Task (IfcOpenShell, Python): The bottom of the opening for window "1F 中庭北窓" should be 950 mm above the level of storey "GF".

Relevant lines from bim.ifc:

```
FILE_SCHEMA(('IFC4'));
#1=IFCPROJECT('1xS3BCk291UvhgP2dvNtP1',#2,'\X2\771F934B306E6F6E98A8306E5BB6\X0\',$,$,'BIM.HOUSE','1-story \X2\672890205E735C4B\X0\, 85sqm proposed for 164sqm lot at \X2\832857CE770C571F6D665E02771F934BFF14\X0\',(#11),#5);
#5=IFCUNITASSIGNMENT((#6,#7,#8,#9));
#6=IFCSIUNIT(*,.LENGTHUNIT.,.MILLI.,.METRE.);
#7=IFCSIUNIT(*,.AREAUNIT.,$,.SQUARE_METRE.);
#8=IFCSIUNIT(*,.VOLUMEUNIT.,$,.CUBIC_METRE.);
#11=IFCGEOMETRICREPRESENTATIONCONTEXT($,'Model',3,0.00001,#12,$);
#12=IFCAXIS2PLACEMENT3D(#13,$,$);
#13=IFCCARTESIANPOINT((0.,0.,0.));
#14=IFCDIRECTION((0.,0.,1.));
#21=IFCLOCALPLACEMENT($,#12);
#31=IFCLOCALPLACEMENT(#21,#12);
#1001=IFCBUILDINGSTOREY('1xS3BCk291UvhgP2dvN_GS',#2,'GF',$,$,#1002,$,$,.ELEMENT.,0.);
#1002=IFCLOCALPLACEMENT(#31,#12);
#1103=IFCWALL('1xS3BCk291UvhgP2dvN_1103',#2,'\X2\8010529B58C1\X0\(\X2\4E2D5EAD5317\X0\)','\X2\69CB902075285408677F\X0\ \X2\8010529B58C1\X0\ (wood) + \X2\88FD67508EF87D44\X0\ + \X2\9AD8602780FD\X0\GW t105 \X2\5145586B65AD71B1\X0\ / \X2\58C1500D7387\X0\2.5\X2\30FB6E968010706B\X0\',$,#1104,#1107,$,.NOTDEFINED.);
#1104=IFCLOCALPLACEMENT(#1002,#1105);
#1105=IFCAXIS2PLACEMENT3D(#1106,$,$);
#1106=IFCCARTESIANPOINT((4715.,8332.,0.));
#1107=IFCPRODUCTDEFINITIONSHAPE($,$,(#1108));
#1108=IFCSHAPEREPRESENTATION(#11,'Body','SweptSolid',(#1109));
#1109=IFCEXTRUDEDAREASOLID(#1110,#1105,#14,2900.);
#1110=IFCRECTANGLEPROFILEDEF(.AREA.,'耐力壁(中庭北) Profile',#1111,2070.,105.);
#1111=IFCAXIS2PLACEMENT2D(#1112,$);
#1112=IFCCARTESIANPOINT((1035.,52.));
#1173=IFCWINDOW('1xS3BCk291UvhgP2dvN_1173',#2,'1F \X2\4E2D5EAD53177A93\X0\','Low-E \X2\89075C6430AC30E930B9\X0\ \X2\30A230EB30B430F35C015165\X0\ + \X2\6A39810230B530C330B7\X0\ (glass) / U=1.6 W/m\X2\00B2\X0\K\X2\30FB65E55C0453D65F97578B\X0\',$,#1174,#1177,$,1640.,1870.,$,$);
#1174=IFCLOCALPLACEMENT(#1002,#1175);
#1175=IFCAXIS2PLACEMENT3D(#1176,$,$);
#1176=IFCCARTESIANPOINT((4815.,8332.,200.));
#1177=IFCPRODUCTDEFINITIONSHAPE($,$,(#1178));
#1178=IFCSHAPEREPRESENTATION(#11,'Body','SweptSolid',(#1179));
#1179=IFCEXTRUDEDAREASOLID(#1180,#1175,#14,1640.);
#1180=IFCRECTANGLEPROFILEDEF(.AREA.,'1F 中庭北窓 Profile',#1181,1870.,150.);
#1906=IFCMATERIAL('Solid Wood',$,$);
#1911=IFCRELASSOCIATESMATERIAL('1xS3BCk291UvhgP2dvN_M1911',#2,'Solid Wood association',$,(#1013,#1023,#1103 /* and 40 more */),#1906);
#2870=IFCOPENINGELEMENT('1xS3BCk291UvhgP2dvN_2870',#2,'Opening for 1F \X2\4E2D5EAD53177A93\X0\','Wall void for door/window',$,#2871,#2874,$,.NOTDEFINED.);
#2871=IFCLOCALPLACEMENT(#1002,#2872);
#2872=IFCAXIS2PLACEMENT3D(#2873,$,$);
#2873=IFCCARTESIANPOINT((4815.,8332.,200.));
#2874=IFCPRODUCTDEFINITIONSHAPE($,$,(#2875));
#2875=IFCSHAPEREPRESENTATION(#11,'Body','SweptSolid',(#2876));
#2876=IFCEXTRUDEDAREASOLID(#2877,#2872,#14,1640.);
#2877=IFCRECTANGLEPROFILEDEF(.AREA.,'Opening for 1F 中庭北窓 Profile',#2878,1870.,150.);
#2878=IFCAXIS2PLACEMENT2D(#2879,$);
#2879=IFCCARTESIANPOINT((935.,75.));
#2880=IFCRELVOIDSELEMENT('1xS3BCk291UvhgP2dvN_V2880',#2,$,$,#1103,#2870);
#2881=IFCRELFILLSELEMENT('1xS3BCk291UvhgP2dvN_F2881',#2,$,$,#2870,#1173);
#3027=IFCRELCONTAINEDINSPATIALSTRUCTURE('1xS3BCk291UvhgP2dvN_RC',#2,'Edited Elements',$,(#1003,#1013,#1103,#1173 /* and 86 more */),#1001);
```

```python
import numpy as np
import ifcopenshell
import ifcopenshell.api.geometry
import ifcopenshell.geom
import ifcopenshell.util.element
import ifcopenshell.util.placement
import ifcopenshell.util.shape
import ifcopenshell.util.unit

model = ifcopenshell.open("bim.ifc")
unit_scale = ifcopenshell.util.unit.calculate_unit_scale(model)

window = model.by_id(1173)
opening = window.FillsVoids[0].RelatingOpeningElement
storey = ifcopenshell.util.element.get_container(window, ifc_class="IfcBuildingStorey")
level = ifcopenshell.util.placement.get_local_placement(storey.ObjectPlacement)[2, 3]

# The opening's origin need not be at the sill, so measure its lowest point.
shape = ifcopenshell.geom.create_shape(ifcopenshell.geom.settings(), opening)
bottom = ifcopenshell.util.shape.get_shape_bottom_elevation(shape, shape.geometry) / unit_scale
dz = level + 0.95 / unit_scale - bottom

shift = np.array([0.0, 0.0, dz])
# The window is not placed relative to its opening, so move both.
for product in (opening, window):
    matrix = ifcopenshell.util.placement.get_local_placement(product.ObjectPlacement)
    matrix[:3, 3] += shift
    ifcopenshell.api.geometry.edit_object_placement(model, product=product, matrix=matrix, is_si=False)

print(f"moved by {dz * unit_scale:+.3f} m")

model.write("bim_updated.ifc")
```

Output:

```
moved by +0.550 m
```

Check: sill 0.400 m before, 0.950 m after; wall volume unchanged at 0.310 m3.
